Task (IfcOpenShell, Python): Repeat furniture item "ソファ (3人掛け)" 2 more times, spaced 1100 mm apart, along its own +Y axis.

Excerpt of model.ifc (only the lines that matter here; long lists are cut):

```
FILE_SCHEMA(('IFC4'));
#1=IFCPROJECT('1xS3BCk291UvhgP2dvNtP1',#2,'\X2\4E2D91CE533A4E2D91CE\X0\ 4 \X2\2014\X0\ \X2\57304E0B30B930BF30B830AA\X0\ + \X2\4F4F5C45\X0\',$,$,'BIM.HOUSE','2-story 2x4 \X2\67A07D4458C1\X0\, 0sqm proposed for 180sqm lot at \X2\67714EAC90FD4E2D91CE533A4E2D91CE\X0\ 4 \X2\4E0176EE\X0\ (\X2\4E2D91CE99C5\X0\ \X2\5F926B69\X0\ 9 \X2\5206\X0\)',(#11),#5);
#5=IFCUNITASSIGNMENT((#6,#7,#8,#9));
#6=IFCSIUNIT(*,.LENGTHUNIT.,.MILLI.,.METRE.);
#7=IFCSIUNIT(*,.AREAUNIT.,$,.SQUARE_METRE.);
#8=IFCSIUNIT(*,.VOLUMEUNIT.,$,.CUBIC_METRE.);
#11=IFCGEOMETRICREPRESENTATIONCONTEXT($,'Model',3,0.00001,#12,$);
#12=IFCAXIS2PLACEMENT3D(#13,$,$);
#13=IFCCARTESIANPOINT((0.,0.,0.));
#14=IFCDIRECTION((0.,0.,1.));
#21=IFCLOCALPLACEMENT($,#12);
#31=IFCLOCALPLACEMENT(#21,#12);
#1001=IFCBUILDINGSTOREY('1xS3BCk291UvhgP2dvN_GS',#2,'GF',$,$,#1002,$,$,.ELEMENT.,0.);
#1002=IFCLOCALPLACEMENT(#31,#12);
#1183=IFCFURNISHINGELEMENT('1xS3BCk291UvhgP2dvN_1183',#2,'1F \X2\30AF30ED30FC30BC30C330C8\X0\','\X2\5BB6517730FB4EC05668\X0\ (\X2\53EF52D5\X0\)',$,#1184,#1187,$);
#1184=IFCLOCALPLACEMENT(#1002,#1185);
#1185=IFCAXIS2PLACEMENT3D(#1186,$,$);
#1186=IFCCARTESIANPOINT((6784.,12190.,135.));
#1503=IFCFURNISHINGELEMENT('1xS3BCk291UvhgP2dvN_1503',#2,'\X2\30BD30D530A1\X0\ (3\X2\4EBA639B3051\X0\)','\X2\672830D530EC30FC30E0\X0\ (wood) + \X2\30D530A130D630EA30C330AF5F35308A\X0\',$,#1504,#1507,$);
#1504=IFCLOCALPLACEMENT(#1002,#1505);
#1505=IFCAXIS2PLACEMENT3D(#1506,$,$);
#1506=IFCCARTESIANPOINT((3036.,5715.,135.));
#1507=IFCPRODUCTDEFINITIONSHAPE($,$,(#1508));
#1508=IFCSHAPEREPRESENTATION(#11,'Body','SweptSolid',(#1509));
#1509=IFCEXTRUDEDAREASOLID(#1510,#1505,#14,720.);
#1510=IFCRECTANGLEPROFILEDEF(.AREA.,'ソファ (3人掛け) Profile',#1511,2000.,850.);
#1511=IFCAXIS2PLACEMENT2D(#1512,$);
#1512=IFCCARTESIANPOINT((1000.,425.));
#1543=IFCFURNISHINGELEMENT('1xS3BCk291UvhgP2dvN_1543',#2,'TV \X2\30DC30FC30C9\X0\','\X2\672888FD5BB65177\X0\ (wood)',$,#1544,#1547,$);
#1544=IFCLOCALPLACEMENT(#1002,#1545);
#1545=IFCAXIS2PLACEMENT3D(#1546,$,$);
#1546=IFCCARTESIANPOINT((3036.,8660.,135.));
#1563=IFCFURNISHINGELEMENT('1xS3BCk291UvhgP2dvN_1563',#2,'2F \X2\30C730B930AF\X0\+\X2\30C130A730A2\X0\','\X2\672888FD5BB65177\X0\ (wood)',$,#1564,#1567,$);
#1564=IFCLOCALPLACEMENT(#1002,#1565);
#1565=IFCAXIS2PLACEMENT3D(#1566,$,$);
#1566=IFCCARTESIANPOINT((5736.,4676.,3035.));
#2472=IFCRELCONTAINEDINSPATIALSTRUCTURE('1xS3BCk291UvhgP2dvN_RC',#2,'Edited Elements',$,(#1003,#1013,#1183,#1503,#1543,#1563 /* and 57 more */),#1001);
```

```python
import ifcopenshell
import ifcopenshell.api.geometry
import ifcopenshell.api.root
import ifcopenshell.util.element
import ifcopenshell.util.placement
import ifcopenshell.util.unit

model = ifcopenshell.open("model.ifc")
unit_scale = ifcopenshell.util.unit.calculate_unit_scale(model)


def reuse_history(source, copy):
    """copy_class also copies each property set's owner history, people and application; keep the originals."""
    for rel in copy.IsDefinedBy:
        if rel.is_a("IfcRelDefinesByProperties") and (history := rel.RelatingPropertyDefinition.OwnerHistory):
            rel.RelatingPropertyDefinition.OwnerHistory = source.OwnerHistory
            ifcopenshell.util.element.remove_deep2(model, history)


source = model.by_guid("1xS3BCk291UvhgP2dvN_1503")
base = ifcopenshell.util.placement.get_local_placement(source.ObjectPlacement)
step = base[:3, 1] * 1.1 / unit_scale

for i in range(1, 3):
    copy = ifcopenshell.api.root.copy_class(model, product=source)
    copy.Representation = ifcopenshell.util.element.copy_deep(
        model, source.Representation, exclude=["IfcGeometricRepresentationContext", "IfcRepresentationMap"]
    )
    reuse_history(source, copy)
    matrix = base.copy()
    matrix[:3, 3] += i * step
    print("added at", matrix[:3, 3].round(3) + 0.0)
    ifcopenshell.api.geometry.edit_object_placement(model, product=copy, matrix=matrix, is_si=False)

model.write("model_v2.ifc")
```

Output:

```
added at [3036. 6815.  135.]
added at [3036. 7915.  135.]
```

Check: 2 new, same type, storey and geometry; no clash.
